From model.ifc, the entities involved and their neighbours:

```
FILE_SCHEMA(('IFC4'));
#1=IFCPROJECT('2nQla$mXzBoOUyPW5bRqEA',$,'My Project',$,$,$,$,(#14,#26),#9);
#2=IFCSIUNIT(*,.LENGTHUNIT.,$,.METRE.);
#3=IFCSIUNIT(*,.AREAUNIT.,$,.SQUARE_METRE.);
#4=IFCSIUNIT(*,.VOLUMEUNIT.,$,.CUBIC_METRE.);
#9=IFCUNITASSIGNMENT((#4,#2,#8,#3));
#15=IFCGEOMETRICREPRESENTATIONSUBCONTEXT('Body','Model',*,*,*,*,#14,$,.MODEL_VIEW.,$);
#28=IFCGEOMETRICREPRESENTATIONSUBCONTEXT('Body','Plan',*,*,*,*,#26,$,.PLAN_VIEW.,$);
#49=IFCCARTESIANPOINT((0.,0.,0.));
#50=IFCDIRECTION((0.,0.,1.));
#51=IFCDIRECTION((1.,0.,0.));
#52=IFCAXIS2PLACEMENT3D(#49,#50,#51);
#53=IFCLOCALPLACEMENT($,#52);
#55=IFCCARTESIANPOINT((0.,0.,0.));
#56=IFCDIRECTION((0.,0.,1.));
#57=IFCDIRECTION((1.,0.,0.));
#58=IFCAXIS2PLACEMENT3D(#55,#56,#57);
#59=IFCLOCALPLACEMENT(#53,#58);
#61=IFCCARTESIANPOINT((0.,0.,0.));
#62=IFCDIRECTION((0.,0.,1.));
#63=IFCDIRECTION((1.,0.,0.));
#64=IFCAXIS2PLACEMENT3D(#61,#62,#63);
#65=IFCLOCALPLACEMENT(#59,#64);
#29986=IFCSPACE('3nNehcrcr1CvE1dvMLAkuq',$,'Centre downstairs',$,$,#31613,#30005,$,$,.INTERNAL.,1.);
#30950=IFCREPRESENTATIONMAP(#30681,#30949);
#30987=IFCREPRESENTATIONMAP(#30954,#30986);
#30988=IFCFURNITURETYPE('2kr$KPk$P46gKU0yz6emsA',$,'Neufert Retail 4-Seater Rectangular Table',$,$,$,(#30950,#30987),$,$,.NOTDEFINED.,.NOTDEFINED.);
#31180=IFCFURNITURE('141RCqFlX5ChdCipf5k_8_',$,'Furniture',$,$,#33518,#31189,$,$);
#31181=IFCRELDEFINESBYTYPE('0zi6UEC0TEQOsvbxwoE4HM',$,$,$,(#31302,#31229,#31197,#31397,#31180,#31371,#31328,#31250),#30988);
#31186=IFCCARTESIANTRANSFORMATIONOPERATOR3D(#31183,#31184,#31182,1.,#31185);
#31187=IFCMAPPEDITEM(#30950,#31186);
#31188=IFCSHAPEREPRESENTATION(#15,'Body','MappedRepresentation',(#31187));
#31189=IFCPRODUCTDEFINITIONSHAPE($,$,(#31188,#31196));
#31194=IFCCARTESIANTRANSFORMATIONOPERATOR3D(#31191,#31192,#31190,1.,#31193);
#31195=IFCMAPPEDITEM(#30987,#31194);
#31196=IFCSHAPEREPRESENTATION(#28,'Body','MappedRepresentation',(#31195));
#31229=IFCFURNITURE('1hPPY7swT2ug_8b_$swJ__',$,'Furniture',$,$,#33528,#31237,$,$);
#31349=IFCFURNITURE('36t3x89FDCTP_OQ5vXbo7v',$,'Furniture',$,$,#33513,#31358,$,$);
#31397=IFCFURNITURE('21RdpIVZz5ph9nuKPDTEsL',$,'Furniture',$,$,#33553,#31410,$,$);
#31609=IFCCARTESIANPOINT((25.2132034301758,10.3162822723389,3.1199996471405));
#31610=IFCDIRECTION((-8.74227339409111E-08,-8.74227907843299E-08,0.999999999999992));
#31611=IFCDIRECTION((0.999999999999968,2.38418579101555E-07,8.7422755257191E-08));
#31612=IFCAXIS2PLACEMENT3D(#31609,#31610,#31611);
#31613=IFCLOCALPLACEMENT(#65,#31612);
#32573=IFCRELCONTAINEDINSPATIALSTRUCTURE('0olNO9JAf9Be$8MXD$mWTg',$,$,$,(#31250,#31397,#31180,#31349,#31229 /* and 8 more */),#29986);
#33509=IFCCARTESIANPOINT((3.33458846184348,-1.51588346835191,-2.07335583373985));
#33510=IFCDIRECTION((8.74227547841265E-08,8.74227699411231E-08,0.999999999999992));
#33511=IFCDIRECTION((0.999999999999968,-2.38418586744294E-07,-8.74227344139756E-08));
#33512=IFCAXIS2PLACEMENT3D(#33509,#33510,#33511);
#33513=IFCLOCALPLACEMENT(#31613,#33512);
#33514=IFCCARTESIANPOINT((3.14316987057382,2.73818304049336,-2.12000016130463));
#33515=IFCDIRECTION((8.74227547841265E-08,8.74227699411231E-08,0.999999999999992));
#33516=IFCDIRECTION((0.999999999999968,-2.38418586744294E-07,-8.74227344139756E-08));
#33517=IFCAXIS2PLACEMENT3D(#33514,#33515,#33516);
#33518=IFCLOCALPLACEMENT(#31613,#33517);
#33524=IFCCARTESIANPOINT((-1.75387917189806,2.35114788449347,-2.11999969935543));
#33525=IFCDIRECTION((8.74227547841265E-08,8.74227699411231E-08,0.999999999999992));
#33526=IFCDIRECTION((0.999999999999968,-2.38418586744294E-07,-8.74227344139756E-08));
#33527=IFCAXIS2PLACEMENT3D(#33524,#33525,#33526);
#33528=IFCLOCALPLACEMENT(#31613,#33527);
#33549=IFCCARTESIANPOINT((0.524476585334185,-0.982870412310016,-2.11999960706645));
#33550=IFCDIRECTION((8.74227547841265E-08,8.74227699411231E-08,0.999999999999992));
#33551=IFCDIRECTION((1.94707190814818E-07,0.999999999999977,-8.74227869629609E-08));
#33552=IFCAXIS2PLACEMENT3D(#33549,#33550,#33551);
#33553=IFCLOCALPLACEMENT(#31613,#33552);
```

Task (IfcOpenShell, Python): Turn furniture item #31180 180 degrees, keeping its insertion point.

```python
import ifcopenshell
import ifcopenshell.api.geometry
import ifcopenshell.util.placement

model = ifcopenshell.open("model.ifc")

item = model.by_guid("141RCqFlX5ChdCipf5k_8_")
matrix = ifcopenshell.util.placement.get_local_placement(item.ObjectPlacement)
matrix = matrix @ ifcopenshell.util.placement.rotation(180, "Z")
ifcopenshell.api.geometry.edit_object_placement(model, product=item, matrix=matrix, is_si=False)

print(ifcopenshell.util.placement.get_local_placement(item.ObjectPlacement).round(3) + 0.0)

model.write("model_edited.ifc")
```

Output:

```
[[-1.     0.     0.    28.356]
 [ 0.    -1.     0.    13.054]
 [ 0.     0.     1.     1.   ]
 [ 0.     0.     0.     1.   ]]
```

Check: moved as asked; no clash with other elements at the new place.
